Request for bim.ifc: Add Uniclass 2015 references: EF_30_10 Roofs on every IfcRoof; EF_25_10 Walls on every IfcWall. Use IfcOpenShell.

First a look at what the model holds.

```python
import ifcopenshell

model = ifcopenshell.open("bim.ifc")
print(model.schema)
print("classifications:", [c.Name for c in model.by_type("IfcClassification")])
for ifc_class in ("IfcDoor", "IfcRoof", "IfcStair", "IfcWall", "IfcWindow"):
    print(ifc_class, len(model.by_type(ifc_class)))
```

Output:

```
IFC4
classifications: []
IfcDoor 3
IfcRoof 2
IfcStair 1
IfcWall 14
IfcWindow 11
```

```python
import ifcopenshell
import ifcopenshell.api.classification

model = ifcopenshell.open("bim.ifc")

system = ifcopenshell.api.classification.add_classification(model, classification="Uniclass 2015")

codes = {
    "IfcRoof": ("EF_30_10", "Roofs"),
    "IfcWall": ("EF_25_10", "Walls"),
}
for ifc_class, (code, name) in codes.items():
    products = model.by_type(ifc_class)
    ifcopenshell.api.classification.add_reference(
        model, products=products, classification=system, identification=code, name=name
    )
    print(code, len(products))

model.write("bim_updated.ifc")
```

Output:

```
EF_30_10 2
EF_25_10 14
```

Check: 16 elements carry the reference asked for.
